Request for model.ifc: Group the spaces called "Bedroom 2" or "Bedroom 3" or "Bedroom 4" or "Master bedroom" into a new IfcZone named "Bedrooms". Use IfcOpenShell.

First a look at what the model holds.

```python
import ifcopenshell

model = ifcopenshell.open("model.ifc")
print(model.schema)
seen = {}
for space in model.by_type("IfcSpace"):
    seen[space.LongName] = seen.get(space.LongName, 0) + 1
for name, count in sorted(seen.items(), key=str):
    print(count, "x", name)
print("zones:", [z.Name for z in model.by_type("IfcZone")][:20])
```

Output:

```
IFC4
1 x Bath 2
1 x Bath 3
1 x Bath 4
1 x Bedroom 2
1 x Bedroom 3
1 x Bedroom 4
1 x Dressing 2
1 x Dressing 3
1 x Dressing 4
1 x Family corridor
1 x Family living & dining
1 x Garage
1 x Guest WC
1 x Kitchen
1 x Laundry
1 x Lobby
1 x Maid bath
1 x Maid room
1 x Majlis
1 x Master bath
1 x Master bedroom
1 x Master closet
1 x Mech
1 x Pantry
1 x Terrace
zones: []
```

```python
import ifcopenshell
import ifcopenshell.api.group
import ifcopenshell.api.root

model = ifcopenshell.open("model.ifc")

names = {"Bedroom 2", "Bedroom 3", "Bedroom 4", "Master bedroom"}
spaces = [s for s in model.by_type("IfcSpace") if s.LongName in names]

zone = ifcopenshell.api.root.create_entity(model, ifc_class="IfcZone", name="Bedrooms")
ifcopenshell.api.group.assign_group(model, products=spaces, group=zone)
print(len(spaces), "spaces in", zone.Name)

model.write("model_rev.ifc")
```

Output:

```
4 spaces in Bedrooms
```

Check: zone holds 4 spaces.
